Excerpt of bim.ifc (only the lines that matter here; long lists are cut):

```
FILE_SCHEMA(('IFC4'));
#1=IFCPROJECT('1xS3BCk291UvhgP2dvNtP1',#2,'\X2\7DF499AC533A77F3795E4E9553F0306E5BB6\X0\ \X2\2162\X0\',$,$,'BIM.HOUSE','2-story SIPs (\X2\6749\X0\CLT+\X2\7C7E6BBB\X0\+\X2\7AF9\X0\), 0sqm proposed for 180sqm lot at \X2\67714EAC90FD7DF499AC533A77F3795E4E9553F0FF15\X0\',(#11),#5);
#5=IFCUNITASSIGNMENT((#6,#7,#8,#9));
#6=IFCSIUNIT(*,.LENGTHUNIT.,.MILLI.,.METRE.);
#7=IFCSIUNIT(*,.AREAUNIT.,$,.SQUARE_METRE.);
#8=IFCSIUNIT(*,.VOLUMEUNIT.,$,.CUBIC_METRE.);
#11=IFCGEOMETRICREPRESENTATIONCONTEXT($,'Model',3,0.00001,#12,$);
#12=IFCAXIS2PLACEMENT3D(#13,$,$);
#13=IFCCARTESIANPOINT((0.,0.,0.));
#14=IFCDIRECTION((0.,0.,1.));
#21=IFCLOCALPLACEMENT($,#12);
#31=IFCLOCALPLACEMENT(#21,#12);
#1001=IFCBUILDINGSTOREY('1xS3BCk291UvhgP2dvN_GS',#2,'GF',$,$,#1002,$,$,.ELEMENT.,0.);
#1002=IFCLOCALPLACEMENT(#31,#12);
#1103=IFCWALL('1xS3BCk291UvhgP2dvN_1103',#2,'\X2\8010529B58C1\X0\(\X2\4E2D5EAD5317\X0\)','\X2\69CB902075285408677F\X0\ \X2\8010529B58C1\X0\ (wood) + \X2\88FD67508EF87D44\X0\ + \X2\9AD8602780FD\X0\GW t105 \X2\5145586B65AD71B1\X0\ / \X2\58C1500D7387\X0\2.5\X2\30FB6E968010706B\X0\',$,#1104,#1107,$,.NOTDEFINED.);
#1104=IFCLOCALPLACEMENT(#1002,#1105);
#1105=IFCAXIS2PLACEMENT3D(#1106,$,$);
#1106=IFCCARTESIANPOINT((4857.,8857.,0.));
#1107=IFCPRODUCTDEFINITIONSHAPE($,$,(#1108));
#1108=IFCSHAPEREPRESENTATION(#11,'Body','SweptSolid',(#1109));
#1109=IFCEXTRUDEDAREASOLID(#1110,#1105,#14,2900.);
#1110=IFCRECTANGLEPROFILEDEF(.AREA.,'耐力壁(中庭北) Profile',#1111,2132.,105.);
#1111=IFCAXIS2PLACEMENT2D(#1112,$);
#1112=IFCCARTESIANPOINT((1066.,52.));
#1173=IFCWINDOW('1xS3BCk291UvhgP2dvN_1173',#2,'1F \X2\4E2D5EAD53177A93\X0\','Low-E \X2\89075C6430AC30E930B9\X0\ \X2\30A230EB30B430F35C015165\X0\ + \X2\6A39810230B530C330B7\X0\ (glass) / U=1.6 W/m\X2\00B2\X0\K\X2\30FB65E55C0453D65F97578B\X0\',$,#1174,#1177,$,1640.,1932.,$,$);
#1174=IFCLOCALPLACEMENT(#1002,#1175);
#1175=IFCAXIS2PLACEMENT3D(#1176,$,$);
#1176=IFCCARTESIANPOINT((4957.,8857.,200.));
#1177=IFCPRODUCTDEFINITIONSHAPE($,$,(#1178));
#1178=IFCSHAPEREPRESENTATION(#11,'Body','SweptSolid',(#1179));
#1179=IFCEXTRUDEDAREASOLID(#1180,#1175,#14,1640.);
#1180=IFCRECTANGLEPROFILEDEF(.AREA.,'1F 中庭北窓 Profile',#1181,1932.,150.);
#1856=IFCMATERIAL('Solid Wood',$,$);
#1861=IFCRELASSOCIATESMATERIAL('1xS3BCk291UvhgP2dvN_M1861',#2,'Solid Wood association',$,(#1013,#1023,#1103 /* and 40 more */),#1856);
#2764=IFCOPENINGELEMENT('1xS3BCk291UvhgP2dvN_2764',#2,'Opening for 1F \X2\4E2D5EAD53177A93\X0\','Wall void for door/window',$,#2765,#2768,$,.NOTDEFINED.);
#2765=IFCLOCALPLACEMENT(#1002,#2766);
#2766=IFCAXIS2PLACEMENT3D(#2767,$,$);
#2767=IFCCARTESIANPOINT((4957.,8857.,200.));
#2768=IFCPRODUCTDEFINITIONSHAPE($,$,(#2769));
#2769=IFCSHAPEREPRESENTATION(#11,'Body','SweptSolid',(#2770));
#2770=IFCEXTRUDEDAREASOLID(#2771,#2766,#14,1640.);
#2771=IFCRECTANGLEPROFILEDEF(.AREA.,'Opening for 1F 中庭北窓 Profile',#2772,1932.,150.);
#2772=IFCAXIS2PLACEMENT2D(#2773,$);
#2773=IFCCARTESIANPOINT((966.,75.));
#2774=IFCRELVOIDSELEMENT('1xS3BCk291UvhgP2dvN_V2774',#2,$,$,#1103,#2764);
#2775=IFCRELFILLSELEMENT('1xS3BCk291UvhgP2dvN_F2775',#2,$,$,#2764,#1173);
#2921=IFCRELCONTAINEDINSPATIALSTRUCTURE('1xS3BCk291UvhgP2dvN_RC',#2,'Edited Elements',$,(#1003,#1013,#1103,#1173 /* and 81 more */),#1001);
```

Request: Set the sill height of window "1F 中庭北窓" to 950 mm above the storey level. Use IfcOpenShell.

```python
import numpy as np
import ifcopenshell
import ifcopenshell.api.geometry
import ifcopenshell.geom
import ifcopenshell.util.element
import ifcopenshell.util.placement
import ifcopenshell.util.shape
import ifcopenshell.util.unit

model = ifcopenshell.open("bim.ifc")
unit_scale = ifcopenshell.util.unit.calculate_unit_scale(model)

window = model.by_guid("1xS3BCk291UvhgP2dvN_1173")
opening = window.FillsVoids[0].RelatingOpeningElement
storey = ifcopenshell.util.element.get_container(window, ifc_class="IfcBuildingStorey")
level = ifcopenshell.util.placement.get_local_placement(storey.ObjectPlacement)[2, 3]

# The opening's origin need not be at the sill, so measure its lowest point.
shape = ifcopenshell.geom.create_shape(ifcopenshell.geom.settings(), opening)
bottom = ifcopenshell.util.shape.get_shape_bottom_elevation(shape, shape.geometry) / unit_scale
dz = level + 0.95 / unit_scale - bottom

shift = np.array([0.0, 0.0, dz])
# The window is not placed relative to its opening, so move both.
for product in (opening, window):
    matrix = ifcopenshell.util.placement.get_local_placement(product.ObjectPlacement)
    matrix[:3, 3] += shift
    ifcopenshell.api.geometry.edit_object_placement(model, product=product, matrix=matrix, is_si=False)

print(f"moved by {dz * unit_scale:+.3f} m")

model.write("bim_edited.ifc")
```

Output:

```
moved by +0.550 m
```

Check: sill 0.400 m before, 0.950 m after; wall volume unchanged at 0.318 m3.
